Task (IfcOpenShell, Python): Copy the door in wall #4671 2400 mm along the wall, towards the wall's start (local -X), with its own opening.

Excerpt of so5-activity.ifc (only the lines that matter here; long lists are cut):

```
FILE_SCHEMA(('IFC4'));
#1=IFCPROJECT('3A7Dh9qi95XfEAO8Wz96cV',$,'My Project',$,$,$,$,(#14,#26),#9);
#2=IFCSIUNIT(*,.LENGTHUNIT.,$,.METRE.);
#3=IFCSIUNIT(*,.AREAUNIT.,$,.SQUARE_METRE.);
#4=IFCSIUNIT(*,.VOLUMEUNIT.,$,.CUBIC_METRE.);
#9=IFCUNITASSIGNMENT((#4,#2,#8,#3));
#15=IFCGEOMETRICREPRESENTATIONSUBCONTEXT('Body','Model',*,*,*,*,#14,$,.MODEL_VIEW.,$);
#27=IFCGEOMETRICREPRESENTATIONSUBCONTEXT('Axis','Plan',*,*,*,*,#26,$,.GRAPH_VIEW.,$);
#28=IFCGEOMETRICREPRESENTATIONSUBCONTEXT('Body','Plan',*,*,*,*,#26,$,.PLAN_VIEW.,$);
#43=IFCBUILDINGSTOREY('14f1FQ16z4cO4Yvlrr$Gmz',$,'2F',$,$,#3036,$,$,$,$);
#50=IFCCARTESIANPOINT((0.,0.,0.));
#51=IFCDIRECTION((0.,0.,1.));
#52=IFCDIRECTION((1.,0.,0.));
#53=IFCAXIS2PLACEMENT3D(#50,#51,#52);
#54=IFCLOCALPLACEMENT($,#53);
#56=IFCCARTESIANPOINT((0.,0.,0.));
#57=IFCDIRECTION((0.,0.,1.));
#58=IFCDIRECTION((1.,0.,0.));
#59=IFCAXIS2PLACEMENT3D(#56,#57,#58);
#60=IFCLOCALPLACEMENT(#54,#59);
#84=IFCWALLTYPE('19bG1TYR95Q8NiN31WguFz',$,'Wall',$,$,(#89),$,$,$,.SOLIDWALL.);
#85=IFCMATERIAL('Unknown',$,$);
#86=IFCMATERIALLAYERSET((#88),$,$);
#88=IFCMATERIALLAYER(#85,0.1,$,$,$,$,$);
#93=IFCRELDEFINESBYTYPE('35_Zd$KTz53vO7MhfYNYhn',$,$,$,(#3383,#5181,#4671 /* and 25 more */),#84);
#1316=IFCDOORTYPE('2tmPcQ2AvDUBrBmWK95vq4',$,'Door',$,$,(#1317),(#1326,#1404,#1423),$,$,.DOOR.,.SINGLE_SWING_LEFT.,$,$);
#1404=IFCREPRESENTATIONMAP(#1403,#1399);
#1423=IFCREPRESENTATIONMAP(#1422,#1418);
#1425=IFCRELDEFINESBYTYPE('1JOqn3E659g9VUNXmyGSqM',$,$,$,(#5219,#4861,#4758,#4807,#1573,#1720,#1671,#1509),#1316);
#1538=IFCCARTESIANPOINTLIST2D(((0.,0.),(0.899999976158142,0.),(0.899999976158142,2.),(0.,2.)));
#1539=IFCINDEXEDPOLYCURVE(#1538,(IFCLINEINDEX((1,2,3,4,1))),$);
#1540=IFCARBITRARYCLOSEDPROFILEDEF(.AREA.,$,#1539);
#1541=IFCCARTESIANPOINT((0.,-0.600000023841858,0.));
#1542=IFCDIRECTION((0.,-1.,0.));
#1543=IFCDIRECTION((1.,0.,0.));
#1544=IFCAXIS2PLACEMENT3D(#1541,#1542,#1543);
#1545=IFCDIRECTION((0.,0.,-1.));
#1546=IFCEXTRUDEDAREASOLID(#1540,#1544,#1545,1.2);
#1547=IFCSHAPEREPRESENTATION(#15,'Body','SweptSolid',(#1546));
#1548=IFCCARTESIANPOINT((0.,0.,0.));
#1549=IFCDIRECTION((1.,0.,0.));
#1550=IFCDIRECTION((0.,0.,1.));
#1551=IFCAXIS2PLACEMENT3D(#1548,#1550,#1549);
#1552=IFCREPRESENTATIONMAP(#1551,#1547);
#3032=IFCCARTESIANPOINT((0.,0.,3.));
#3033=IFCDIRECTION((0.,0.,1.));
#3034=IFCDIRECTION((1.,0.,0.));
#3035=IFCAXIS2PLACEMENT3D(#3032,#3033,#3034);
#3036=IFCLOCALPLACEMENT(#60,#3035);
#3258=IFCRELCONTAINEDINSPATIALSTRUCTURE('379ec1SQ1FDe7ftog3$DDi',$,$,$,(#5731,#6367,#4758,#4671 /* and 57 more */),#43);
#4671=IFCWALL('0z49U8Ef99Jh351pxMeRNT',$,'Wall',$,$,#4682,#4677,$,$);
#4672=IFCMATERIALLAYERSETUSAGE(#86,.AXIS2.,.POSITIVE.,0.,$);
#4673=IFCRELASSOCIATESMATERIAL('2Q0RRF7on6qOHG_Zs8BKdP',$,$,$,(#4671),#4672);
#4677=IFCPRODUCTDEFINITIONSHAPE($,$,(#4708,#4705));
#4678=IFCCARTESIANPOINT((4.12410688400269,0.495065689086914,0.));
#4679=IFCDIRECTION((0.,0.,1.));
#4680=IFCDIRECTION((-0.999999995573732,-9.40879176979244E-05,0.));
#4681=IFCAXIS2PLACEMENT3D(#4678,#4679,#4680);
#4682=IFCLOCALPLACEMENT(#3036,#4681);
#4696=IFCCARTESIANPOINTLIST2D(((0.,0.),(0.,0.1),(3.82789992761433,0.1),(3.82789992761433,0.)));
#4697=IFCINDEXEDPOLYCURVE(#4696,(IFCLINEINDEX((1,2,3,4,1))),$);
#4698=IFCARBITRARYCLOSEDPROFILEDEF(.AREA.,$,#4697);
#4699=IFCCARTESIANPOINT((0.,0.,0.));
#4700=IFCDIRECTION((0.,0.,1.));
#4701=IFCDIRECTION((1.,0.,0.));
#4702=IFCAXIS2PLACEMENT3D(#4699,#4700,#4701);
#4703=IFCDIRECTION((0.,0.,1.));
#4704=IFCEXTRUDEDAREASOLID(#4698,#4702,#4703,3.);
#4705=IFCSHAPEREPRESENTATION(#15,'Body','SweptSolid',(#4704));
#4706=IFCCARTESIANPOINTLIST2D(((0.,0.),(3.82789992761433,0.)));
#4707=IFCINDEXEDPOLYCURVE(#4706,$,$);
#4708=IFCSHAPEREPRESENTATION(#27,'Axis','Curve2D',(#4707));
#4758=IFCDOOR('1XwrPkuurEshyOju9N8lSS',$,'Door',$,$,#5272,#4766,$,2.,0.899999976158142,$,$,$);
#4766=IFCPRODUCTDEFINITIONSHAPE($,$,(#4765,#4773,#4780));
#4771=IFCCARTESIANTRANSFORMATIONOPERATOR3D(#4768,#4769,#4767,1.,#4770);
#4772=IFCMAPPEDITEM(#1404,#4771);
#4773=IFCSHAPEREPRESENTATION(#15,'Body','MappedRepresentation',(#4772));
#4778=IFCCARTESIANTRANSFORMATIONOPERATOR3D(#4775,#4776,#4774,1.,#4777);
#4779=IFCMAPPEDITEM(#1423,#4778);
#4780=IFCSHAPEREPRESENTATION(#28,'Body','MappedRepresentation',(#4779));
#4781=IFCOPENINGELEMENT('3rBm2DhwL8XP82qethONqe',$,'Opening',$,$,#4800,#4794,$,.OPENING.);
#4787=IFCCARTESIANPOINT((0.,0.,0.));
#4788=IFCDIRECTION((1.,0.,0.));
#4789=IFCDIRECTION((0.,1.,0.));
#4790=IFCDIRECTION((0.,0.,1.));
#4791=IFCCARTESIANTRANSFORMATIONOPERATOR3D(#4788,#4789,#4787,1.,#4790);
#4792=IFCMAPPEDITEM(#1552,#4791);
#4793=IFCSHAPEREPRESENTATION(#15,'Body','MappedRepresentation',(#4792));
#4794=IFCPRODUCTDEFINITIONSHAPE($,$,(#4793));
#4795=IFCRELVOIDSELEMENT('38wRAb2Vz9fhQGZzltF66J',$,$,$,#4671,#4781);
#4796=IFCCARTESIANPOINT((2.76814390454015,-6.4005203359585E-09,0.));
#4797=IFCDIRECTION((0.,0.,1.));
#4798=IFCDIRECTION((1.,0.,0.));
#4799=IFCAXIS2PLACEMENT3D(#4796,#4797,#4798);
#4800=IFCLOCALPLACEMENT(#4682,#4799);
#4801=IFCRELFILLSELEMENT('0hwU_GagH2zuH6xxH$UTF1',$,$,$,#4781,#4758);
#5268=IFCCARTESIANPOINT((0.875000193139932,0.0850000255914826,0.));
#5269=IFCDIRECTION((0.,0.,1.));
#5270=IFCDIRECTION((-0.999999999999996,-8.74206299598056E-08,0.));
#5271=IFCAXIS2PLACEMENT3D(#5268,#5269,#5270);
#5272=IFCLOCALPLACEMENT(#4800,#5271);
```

```python
import ifcopenshell
import ifcopenshell.api.feature
import ifcopenshell.api.geometry
import ifcopenshell.api.root
import ifcopenshell.geom
import ifcopenshell.util.element
import ifcopenshell.util.placement
import ifcopenshell.util.shape
import ifcopenshell.util.unit

model = ifcopenshell.open("so5-activity.ifc")
unit_scale = ifcopenshell.util.unit.calculate_unit_scale(model)
settings = ifcopenshell.geom.settings()


def volume(element):
    """Net volume in cubic metres, openings subtracted."""
    shape = ifcopenshell.geom.create_shape(settings, element)
    return ifcopenshell.util.shape.get_volume(shape.geometry)


door = model.by_guid("1XwrPkuurEshyOju9N8lSS")
opening = door.FillsVoids[0].RelatingOpeningElement
wall = opening.VoidsElements[0].RelatingBuildingElement
before = volume(wall)
shift = ifcopenshell.util.placement.get_local_placement(wall.ObjectPlacement)[:3, 0] * -2.4 / unit_scale

# copy_class copies the void relationship, type, container and properties, but no geometry.
new_opening = ifcopenshell.api.root.copy_class(model, product=opening)
new_opening.Representation = ifcopenshell.util.element.copy_deep(
    model, opening.Representation, exclude=["IfcGeometricRepresentationContext", "IfcRepresentationMap"]
)
new_door = ifcopenshell.api.root.copy_class(model, product=door)
new_door.Representation = ifcopenshell.util.element.copy_deep(
    model, door.Representation, exclude=["IfcGeometricRepresentationContext", "IfcRepresentationMap"]
)
ifcopenshell.api.feature.add_filling(model, opening=new_opening, element=new_door)

for old, new in ((opening, new_opening), (door, new_door)):
    matrix = ifcopenshell.util.placement.get_local_placement(old.ObjectPlacement)
    matrix[:3, 3] += shift
    ifcopenshell.api.geometry.edit_object_placement(model, product=new, matrix=matrix, is_si=False)

after = volume(wall)

print(f"wall volume {before:.3f} -> {after:.3f} m3")

model.write("so5-activity_updated.ifc")
```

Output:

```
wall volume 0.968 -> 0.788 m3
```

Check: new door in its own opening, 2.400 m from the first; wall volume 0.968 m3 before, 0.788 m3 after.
